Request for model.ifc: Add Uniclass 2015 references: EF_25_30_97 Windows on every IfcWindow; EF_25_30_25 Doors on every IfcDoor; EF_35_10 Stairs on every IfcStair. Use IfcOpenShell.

First a look at what the model holds.

```python
import ifcopenshell

model = ifcopenshell.open("model.ifc")
print(model.schema)
print("classifications:", [c.Name for c in model.by_type("IfcClassification")])
for ifc_class in ("IfcDoor", "IfcRoof", "IfcStair", "IfcWall", "IfcWindow"):
    print(ifc_class, len(model.by_type(ifc_class)))
```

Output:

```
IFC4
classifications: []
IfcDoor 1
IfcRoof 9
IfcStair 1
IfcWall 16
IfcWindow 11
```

```python
import ifcopenshell
import ifcopenshell.api.classification

model = ifcopenshell.open("model.ifc")

system = ifcopenshell.api.classification.add_classification(model, classification="Uniclass 2015")

codes = {
    "IfcWindow": ("EF_25_30_97", "Windows"),
    "IfcDoor": ("EF_25_30_25", "Doors"),
    "IfcStair": ("EF_35_10", "Stairs"),
}
for ifc_class, (code, name) in codes.items():
    products = model.by_type(ifc_class)
    ifcopenshell.api.classification.add_reference(
        model, products=products, classification=system, identification=code, name=name
    )
    print(code, len(products))

model.write("model_v2.ifc")
```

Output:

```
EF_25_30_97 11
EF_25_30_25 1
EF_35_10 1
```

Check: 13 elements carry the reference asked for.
